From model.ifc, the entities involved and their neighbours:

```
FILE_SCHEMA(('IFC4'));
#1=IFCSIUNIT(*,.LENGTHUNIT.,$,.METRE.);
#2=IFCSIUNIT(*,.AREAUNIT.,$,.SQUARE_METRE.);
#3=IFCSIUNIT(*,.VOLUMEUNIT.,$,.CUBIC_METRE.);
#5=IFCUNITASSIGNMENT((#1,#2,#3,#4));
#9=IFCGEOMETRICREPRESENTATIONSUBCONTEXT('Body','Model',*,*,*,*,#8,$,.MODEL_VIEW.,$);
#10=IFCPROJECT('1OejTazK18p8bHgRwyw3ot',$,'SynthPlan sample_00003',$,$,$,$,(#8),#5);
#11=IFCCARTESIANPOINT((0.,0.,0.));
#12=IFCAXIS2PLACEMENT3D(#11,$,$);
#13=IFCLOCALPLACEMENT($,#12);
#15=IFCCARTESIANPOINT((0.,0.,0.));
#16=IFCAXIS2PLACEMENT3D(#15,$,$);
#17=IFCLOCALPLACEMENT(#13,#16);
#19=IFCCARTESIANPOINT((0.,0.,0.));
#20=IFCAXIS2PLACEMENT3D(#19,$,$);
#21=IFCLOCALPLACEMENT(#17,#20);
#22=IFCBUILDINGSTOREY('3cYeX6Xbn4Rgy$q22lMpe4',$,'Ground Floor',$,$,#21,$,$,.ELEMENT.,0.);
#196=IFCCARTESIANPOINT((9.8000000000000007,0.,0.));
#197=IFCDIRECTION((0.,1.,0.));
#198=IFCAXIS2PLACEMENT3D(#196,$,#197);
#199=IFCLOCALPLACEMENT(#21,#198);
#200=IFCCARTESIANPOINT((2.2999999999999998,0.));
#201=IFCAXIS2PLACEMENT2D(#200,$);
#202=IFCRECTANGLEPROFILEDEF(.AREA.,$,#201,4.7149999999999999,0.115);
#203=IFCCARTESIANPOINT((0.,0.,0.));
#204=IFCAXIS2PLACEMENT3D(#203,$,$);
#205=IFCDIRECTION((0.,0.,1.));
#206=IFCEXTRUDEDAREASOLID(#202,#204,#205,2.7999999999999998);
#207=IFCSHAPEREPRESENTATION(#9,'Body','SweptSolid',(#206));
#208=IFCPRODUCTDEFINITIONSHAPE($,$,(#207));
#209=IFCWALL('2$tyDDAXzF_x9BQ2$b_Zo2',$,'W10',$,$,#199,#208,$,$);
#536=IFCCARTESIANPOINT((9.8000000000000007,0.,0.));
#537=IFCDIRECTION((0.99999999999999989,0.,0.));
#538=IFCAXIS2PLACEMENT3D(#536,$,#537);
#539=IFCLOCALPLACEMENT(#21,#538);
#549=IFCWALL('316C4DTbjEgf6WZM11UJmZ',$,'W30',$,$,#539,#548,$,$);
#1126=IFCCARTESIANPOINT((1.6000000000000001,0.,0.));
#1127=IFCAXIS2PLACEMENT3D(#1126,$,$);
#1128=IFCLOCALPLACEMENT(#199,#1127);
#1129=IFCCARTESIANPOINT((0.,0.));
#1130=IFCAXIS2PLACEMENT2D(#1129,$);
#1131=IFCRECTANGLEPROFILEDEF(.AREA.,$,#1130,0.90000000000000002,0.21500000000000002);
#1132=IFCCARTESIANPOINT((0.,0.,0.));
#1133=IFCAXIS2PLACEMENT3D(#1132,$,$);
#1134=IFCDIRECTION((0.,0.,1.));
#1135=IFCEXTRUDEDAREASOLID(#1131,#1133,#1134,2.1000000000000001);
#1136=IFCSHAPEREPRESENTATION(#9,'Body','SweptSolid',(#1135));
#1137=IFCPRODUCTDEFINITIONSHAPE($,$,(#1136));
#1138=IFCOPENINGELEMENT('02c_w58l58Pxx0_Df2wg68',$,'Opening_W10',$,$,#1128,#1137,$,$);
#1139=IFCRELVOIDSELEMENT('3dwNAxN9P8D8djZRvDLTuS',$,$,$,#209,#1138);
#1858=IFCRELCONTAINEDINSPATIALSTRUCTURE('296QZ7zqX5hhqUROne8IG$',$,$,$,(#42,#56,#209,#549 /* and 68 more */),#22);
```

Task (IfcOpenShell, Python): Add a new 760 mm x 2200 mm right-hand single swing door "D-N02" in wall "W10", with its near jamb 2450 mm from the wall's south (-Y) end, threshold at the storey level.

```python
import numpy as np
import ifcopenshell
import ifcopenshell.api.feature
import ifcopenshell.api.geometry
import ifcopenshell.api.root
import ifcopenshell.api.spatial
import ifcopenshell.geom
import ifcopenshell.util.element
import ifcopenshell.util.placement
import ifcopenshell.util.representation
import ifcopenshell.util.shape
import ifcopenshell.util.unit

model = ifcopenshell.open("model.ifc")
unit_scale = ifcopenshell.util.unit.calculate_unit_scale(model)
settings = ifcopenshell.geom.settings()


def volume(element):
    """Net volume in cubic metres, openings subtracted."""
    shape = ifcopenshell.geom.create_shape(settings, element)
    return ifcopenshell.util.shape.get_volume(shape.geometry)


wall = model.by_id(209)
storey = ifcopenshell.util.element.get_container(wall, ifc_class="IfcBuildingStorey")
context = ifcopenshell.util.representation.get_context(model, "Model", "Body", "MODEL_VIEW")
before = volume(wall)

width, height, from_end, sill = 0.76, 2.2, 2.45, 0.0  # metres

# The wall runs along its own X axis, and the end named is its -X end.
wall_shape = ifcopenshell.geom.create_shape(settings, wall)
x, y, z = ifcopenshell.util.shape.get_vertices(wall_shape.geometry).T
start = x.min() + from_end
face, thickness = float(y.min()), float(y.max() - y.min())
wall_matrix = ifcopenshell.util.placement.get_local_placement(wall.ObjectPlacement)
level = ifcopenshell.util.placement.get_local_placement(storey.ObjectPlacement)[2, 3]


def in_wall(x, y):
    """Placement at x, y metres in the wall's axes, at sill height."""
    matrix = wall_matrix.copy()
    matrix[:, 3] = wall_matrix @ np.array([x / unit_scale, y / unit_scale, 0.0, 1.0])
    matrix[2, 3] = level + sill / unit_scale
    return matrix


# Opening: a box that overshoots both wall faces by 50 mm.
opening = ifcopenshell.api.root.create_entity(model, ifc_class="IfcOpeningElement", predefined_type="OPENING")
box = ifcopenshell.api.geometry.add_wall_representation(
    model, context=context, length=width, height=height, thickness=thickness + 0.1
)
ifcopenshell.api.geometry.assign_representation(model, product=opening, representation=box)
ifcopenshell.api.geometry.edit_object_placement(model, product=opening, matrix=in_wall(start, face - 0.05), is_si=False)
ifcopenshell.api.feature.add_feature(model, feature=opening, element=wall)

door = ifcopenshell.api.root.create_entity(model, ifc_class="IfcDoor", name="D-N02", predefined_type="DOOR")
door.OverallWidth, door.OverallHeight = width / unit_scale, height / unit_scale
door.OperationType = "SINGLE_SWING_RIGHT"
body = ifcopenshell.api.geometry.add_door_representation(
    model,
    context=context,
    overall_width=door.OverallWidth,
    overall_height=door.OverallHeight,
    operation_type="SINGLE_SWING_RIGHT",
    lining_properties={"LiningDepth": thickness / unit_scale, "ThresholdDepth": thickness / unit_scale},
)
ifcopenshell.api.geometry.assign_representation(model, product=door, representation=body)
ifcopenshell.api.spatial.assign_container(model, products=[door], relating_structure=storey)
ifcopenshell.api.feature.add_filling(model, opening=opening, element=door)

# The lining spans the wall, so the door starts at the wall face.
ifcopenshell.api.geometry.edit_object_placement(model, product=door, matrix=in_wall(start, face), is_si=False)

after = volume(wall)

print(f"wall volume {before:.3f} -> {after:.3f} m3")

model.write("model_rev.ifc")
```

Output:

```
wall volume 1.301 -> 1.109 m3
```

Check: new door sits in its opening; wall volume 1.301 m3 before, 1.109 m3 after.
